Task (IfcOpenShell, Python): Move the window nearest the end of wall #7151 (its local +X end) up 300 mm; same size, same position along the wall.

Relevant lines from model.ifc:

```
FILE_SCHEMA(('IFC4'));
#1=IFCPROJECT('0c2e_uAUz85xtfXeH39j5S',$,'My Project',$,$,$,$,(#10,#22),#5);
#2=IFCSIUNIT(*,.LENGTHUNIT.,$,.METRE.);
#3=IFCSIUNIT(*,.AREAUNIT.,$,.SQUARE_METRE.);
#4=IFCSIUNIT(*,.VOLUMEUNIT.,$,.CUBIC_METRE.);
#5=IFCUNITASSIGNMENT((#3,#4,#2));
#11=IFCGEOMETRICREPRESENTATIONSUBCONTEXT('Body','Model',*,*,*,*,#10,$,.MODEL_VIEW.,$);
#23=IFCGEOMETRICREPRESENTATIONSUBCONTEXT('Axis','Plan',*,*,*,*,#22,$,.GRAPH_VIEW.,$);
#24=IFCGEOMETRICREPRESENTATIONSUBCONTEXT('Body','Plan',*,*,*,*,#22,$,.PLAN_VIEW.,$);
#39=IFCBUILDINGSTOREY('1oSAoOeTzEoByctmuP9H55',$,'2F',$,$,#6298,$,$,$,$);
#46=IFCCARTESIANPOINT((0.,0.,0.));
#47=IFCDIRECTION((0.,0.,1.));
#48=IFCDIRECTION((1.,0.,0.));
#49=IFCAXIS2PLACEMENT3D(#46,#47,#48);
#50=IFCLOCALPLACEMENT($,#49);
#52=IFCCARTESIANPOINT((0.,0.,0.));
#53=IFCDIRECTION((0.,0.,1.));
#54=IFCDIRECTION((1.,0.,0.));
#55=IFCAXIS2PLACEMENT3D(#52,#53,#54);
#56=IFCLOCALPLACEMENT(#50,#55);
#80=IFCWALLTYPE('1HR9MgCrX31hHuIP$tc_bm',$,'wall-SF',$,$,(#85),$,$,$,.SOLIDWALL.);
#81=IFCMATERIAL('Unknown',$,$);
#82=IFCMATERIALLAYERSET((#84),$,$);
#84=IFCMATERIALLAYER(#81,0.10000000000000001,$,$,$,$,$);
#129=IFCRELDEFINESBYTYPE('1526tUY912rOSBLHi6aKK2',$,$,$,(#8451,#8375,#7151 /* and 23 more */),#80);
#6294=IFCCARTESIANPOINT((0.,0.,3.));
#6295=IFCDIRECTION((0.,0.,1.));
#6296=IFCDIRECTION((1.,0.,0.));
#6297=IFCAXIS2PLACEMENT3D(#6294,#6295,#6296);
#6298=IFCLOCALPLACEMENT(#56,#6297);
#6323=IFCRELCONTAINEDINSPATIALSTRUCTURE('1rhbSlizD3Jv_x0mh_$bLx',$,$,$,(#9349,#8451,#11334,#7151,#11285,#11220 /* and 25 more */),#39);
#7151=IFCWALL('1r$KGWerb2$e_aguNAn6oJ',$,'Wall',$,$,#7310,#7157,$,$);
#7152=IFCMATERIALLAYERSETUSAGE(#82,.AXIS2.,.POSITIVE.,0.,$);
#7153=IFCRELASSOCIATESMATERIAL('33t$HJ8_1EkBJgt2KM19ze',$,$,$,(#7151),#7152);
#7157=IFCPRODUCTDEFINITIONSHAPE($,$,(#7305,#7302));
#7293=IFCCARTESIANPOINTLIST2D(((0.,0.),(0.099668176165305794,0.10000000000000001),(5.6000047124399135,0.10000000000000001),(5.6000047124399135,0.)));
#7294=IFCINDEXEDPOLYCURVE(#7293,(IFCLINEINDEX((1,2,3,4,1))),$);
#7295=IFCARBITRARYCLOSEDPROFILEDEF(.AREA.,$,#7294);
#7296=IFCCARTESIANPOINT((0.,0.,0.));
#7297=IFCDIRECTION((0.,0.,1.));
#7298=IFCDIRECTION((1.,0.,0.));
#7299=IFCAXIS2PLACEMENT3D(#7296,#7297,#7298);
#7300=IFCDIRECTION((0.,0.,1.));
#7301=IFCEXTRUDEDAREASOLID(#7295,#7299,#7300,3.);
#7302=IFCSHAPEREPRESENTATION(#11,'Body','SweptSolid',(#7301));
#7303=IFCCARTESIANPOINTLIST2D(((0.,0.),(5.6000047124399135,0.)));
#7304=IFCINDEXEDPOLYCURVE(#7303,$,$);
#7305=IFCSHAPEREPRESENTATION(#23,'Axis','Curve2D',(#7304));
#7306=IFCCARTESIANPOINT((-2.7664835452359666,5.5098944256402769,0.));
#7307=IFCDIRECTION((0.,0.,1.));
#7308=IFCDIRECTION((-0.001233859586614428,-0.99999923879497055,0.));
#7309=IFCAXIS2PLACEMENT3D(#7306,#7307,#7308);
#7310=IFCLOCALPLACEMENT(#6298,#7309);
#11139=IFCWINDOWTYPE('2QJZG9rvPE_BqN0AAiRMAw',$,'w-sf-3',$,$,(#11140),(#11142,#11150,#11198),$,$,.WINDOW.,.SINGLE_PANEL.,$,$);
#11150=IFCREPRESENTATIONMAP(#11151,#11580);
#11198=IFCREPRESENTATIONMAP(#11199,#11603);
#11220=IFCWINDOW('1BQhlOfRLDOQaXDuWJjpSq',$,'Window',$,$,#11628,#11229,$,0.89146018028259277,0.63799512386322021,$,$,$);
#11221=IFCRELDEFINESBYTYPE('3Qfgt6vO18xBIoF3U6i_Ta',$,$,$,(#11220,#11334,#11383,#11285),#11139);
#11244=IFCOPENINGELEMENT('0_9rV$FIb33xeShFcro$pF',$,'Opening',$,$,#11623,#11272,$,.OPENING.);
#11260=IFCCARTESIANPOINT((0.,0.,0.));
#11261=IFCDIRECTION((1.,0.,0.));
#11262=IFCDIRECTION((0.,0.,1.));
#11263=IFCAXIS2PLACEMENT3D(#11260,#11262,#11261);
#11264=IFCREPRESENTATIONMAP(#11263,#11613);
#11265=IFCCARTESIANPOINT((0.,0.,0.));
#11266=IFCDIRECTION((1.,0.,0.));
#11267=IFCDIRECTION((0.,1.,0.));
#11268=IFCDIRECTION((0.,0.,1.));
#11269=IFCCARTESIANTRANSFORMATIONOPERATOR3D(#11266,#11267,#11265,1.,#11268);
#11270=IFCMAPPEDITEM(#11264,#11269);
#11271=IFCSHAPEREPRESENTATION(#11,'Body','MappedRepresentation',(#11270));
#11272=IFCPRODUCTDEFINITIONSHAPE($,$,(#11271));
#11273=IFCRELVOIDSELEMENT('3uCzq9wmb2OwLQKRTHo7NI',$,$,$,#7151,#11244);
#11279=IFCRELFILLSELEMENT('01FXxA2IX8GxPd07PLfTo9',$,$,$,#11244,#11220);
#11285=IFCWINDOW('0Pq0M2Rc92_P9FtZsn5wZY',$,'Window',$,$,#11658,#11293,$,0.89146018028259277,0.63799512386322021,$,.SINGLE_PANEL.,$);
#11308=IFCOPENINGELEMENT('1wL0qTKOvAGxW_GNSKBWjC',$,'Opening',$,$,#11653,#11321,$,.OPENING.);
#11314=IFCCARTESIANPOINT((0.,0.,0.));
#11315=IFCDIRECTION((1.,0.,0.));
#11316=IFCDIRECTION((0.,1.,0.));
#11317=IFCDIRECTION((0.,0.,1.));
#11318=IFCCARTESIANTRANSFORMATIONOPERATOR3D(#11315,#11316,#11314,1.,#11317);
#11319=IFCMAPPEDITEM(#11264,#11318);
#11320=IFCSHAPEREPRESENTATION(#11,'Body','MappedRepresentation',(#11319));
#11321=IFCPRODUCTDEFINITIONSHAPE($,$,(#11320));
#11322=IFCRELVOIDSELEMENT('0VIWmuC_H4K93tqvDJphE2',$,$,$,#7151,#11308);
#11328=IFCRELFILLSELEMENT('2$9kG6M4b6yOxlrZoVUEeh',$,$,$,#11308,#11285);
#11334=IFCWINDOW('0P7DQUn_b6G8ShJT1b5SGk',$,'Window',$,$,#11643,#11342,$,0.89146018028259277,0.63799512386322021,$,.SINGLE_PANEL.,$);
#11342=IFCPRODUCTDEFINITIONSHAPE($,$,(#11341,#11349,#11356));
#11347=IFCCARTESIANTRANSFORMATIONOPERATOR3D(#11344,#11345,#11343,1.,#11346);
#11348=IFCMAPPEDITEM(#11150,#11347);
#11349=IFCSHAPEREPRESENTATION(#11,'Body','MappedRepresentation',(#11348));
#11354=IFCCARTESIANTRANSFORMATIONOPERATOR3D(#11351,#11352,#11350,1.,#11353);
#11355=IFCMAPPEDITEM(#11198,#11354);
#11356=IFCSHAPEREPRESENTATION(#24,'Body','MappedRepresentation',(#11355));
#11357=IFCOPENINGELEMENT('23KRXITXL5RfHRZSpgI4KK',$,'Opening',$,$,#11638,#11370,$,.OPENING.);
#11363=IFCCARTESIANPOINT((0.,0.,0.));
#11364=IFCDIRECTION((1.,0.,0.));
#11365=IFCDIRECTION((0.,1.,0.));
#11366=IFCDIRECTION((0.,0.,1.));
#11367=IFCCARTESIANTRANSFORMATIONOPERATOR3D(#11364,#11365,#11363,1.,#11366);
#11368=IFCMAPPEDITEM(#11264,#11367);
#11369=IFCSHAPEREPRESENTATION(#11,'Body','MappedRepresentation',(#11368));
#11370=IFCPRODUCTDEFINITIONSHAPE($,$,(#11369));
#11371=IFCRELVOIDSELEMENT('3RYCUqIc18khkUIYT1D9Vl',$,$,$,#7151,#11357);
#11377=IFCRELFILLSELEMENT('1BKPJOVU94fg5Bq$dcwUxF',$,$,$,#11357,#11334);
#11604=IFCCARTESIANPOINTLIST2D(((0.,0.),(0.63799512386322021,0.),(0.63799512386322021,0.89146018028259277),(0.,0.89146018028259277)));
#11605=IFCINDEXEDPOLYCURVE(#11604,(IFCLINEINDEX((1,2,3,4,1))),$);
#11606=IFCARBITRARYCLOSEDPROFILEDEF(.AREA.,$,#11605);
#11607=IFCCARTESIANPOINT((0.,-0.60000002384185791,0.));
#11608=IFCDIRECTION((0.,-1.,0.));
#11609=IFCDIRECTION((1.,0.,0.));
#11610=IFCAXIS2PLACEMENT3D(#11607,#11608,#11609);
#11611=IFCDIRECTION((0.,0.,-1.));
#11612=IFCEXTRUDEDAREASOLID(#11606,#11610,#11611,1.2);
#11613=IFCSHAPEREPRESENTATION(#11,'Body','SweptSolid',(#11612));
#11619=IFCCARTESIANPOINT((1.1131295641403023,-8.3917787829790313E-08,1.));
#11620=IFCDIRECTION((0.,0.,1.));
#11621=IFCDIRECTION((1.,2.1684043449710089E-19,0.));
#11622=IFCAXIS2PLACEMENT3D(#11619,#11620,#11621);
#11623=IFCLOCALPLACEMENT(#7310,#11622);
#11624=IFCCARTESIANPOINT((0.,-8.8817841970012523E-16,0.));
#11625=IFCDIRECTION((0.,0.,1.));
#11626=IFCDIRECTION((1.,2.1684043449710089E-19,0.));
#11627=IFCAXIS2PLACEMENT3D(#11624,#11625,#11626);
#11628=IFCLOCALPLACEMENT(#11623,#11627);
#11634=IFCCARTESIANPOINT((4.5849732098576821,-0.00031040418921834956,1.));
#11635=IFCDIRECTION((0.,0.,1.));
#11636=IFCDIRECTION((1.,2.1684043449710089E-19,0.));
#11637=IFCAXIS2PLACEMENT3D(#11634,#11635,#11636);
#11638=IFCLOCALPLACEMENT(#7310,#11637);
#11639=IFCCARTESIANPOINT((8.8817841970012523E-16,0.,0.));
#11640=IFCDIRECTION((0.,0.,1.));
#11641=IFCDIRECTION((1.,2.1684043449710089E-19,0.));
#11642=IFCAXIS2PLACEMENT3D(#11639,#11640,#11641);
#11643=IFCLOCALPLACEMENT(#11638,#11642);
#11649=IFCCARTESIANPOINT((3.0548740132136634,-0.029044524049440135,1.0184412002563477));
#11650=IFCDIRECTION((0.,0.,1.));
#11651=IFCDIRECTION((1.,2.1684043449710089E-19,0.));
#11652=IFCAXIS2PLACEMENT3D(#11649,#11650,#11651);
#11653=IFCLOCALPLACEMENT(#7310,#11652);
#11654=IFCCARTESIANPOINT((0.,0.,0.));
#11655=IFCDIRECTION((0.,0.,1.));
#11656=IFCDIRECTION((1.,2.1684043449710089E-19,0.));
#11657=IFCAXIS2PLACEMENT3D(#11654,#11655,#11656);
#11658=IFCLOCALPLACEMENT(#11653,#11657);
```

```python
import numpy as np
import ifcopenshell
import ifcopenshell.api.geometry
import ifcopenshell.util.placement
import ifcopenshell.util.unit

model = ifcopenshell.open("model.ifc")
unit_scale = ifcopenshell.util.unit.calculate_unit_scale(model)

window = model.by_guid("0P7DQUn_b6G8ShJT1b5SGk")
opening = window.FillsVoids[0].RelatingOpeningElement
dz = 0.3 / unit_scale

shift = np.array([0.0, 0.0, dz])
# The window is placed relative to its opening, so it follows when the opening moves.
matrix = ifcopenshell.util.placement.get_local_placement(opening.ObjectPlacement)
matrix[:3, 3] += shift
ifcopenshell.api.geometry.edit_object_placement(
    model, product=opening, matrix=matrix, is_si=False, should_transform_children=True
)

print(f"moved by {dz * unit_scale:+.3f} m")

model.write("model-out.ifc")
```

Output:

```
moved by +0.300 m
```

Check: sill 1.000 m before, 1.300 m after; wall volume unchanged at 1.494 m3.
